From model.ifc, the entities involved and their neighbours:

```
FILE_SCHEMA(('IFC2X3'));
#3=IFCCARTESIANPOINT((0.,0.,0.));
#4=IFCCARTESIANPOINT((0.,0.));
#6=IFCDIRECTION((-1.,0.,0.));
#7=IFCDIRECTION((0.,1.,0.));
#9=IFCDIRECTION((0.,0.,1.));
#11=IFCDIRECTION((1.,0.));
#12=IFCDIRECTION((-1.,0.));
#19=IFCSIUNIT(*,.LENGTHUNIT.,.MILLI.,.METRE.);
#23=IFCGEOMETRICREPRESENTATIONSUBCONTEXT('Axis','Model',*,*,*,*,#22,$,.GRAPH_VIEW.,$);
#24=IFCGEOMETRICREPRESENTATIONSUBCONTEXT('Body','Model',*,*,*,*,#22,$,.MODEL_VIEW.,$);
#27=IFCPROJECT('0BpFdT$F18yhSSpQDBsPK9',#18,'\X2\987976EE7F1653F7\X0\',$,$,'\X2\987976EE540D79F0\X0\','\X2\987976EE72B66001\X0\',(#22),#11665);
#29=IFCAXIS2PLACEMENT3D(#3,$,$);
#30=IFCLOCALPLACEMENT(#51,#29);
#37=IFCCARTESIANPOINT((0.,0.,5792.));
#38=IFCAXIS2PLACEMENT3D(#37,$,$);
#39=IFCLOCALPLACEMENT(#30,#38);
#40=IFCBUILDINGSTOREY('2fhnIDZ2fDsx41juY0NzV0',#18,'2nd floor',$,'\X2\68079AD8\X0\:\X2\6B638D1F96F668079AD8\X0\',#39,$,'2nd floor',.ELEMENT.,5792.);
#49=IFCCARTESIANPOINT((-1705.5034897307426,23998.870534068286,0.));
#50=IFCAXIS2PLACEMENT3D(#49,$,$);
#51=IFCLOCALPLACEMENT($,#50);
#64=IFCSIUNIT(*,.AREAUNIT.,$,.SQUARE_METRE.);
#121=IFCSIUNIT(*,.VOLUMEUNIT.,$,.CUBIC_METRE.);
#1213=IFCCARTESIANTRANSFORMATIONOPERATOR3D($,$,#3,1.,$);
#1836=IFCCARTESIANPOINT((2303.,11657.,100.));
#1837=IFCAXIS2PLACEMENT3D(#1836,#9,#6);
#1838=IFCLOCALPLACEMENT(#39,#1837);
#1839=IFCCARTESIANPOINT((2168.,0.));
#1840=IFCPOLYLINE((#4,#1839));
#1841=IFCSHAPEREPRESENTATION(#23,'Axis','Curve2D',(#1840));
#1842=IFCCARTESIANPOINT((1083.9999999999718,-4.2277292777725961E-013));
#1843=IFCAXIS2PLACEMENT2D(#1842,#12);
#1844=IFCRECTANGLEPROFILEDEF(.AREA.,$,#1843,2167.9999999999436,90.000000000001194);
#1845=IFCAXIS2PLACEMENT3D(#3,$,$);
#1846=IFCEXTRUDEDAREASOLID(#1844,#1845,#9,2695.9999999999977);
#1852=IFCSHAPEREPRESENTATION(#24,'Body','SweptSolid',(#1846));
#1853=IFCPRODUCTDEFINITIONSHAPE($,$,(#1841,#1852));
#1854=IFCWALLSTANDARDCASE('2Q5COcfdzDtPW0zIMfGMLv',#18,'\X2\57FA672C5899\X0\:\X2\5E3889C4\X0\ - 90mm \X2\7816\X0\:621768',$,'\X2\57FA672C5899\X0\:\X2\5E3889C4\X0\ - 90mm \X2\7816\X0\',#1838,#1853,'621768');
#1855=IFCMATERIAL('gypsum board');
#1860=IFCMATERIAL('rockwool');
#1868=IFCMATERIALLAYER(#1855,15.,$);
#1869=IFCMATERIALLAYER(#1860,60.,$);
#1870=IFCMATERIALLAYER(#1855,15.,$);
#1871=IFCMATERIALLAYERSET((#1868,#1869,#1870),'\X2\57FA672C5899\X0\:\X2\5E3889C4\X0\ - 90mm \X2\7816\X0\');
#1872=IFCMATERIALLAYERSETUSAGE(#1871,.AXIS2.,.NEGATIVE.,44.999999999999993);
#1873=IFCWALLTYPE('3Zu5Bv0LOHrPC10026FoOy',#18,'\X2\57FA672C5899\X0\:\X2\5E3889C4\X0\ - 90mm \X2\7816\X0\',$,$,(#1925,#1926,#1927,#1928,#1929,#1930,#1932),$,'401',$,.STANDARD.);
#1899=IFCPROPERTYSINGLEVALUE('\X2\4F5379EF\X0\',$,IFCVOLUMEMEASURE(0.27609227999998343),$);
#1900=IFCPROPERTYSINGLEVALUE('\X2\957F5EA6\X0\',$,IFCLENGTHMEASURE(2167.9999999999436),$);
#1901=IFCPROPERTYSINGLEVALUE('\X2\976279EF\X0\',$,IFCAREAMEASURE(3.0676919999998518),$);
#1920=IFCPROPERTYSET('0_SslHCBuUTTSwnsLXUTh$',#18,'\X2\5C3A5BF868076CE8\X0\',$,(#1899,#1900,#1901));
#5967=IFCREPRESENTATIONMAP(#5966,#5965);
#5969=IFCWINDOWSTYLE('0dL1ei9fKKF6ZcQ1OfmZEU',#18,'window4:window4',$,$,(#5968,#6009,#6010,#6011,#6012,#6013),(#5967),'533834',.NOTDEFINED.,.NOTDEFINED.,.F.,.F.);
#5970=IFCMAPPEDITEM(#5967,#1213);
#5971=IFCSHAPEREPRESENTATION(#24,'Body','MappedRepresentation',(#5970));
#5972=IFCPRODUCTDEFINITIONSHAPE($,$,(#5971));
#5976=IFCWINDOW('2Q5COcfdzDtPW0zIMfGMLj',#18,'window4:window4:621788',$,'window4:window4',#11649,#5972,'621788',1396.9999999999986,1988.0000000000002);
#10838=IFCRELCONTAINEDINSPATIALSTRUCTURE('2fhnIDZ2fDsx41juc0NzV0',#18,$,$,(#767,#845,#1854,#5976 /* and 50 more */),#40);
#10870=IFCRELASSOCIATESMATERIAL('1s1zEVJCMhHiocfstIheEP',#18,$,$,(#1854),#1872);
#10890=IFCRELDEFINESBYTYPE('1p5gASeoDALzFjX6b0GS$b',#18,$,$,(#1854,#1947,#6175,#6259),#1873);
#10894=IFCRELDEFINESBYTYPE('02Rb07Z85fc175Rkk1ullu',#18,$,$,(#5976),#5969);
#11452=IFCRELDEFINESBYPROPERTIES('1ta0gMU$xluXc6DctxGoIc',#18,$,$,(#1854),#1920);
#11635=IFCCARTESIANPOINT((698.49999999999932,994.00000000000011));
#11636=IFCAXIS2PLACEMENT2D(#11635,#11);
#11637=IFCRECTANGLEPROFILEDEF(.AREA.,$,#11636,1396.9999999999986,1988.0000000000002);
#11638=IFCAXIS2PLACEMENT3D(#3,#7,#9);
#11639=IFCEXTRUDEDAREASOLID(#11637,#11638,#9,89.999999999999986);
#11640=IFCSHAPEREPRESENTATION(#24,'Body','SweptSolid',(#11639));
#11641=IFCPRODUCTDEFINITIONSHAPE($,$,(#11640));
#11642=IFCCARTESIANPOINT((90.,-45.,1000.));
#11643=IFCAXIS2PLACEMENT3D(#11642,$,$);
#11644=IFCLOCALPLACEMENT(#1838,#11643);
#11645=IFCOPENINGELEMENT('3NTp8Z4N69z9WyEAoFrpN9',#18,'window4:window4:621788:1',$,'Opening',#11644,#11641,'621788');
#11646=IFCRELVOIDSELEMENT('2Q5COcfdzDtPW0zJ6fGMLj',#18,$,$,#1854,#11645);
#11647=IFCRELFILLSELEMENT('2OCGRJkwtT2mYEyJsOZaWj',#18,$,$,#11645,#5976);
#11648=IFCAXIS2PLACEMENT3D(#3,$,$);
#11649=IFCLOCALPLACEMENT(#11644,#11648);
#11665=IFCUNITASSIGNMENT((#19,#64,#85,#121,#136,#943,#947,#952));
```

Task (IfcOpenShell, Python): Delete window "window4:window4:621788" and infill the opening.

```python
import ifcopenshell
import ifcopenshell.api.feature
import ifcopenshell.api.pset
import ifcopenshell.api.root
import ifcopenshell.geom
import ifcopenshell.util.element
import ifcopenshell.util.shape
import ifcopenshell.util.unit

model = ifcopenshell.open("model.ifc")
area_scale = ifcopenshell.util.unit.calculate_unit_scale(model, "AREAUNIT")
volume_scale = ifcopenshell.util.unit.calculate_unit_scale(model, "VOLUMEUNIT")
settings = ifcopenshell.geom.settings()


def volume(element):
    """Net volume in cubic metres, openings subtracted."""
    shape = ifcopenshell.geom.create_shape(settings, element)
    return ifcopenshell.util.shape.get_volume(shape.geometry)


window = model.by_guid("2Q5COcfdzDtPW0zIMfGMLj")
opening = window.FillsVoids[0].RelatingOpeningElement
wall = opening.VoidsElements[0].RelatingBuildingElement
before = volume(wall)

ifcopenshell.api.root.remove_product(model, product=window)
ifcopenshell.api.feature.remove_feature(model, feature=opening)

after = volume(wall)
thickness = 0.09  # wall thickness in metres

# Update the wall's stored quantities.
pset = model.by_id(ifcopenshell.util.element.get_pset(wall, "尺寸标注", should_inherit=False)["id"])
ifcopenshell.api.pset.edit_pset(model, pset=pset, properties={
    "体积": model.create_entity("IfcVolumeMeasure", after / volume_scale),
    "面积": model.create_entity("IfcAreaMeasure", after / thickness / area_scale),
})

print(f"wall volume {before:.3f} -> {after:.3f} m3")

model.write("model-out.ifc")
```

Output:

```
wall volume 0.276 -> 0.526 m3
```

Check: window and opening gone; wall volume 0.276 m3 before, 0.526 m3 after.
